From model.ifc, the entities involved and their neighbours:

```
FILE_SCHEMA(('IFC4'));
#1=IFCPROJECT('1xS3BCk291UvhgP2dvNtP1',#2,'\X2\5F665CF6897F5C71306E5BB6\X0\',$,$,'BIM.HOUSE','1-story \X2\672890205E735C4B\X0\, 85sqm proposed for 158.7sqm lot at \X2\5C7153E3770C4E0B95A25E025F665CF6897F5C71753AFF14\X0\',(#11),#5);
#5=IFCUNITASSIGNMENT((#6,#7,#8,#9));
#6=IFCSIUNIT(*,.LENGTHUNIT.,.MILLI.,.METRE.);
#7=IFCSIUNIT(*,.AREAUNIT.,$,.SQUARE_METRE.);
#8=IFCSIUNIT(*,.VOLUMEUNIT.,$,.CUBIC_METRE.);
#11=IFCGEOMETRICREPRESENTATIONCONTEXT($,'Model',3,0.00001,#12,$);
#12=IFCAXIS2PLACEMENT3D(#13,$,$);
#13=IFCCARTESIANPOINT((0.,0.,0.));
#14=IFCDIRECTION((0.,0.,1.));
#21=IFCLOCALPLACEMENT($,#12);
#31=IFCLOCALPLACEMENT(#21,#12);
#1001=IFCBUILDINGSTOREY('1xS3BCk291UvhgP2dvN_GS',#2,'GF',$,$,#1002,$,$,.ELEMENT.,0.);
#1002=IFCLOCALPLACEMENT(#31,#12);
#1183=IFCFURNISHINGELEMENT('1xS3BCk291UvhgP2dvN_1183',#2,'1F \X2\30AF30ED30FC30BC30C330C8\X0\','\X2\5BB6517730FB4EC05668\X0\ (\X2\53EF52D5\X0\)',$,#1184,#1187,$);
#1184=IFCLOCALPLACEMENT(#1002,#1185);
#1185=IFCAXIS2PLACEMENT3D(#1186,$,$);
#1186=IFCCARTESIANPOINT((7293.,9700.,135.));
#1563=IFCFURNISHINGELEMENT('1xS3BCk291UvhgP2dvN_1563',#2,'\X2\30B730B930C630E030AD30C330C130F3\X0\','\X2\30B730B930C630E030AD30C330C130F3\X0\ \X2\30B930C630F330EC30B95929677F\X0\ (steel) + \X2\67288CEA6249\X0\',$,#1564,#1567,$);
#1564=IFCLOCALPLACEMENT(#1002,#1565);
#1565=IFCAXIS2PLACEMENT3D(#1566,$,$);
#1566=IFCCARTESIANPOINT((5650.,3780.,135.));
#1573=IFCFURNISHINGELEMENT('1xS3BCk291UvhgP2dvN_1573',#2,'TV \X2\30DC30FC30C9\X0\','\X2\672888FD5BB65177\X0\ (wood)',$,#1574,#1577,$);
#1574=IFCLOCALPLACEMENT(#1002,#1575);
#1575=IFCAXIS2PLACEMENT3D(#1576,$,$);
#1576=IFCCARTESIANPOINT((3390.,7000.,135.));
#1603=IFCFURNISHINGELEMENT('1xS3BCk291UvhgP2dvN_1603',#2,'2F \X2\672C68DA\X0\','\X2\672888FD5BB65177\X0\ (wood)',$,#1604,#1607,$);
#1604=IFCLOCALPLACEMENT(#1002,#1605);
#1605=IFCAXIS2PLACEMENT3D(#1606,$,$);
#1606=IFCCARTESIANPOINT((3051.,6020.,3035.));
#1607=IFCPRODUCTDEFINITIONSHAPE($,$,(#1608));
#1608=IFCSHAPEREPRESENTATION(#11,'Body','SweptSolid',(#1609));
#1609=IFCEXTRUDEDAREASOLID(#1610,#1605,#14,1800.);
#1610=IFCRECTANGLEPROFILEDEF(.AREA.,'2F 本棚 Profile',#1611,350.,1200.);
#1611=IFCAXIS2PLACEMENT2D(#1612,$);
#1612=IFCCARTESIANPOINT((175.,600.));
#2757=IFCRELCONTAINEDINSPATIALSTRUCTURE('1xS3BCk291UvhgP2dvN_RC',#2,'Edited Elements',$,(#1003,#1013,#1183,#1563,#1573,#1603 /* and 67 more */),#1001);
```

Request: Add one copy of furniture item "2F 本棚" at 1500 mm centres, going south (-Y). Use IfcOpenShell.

```python
import numpy as np
import ifcopenshell
import ifcopenshell.api.geometry
import ifcopenshell.api.root
import ifcopenshell.util.element
import ifcopenshell.util.placement
import ifcopenshell.util.unit

model = ifcopenshell.open("model.ifc")
unit_scale = ifcopenshell.util.unit.calculate_unit_scale(model)


def reuse_history(source, copy):
    """copy_class also copies each property set's owner history, people and application; keep the originals."""
    for rel in copy.IsDefinedBy:
        if rel.is_a("IfcRelDefinesByProperties") and (history := rel.RelatingPropertyDefinition.OwnerHistory):
            rel.RelatingPropertyDefinition.OwnerHistory = source.OwnerHistory
            ifcopenshell.util.element.remove_deep2(model, history)


source = model.by_guid("1xS3BCk291UvhgP2dvN_1603")
base = ifcopenshell.util.placement.get_local_placement(source.ObjectPlacement)
step = np.array([0.0, -1.0, 0.0]) * 1.5 / unit_scale

for i in range(1, 2):
    copy = ifcopenshell.api.root.copy_class(model, product=source)
    copy.Representation = ifcopenshell.util.element.copy_deep(
        model, source.Representation, exclude=["IfcGeometricRepresentationContext", "IfcRepresentationMap"]
    )
    reuse_history(source, copy)
    matrix = base.copy()
    matrix[:3, 3] += i * step
    print("added at", matrix[:3, 3].round(3) + 0.0)
    ifcopenshell.api.geometry.edit_object_placement(model, product=copy, matrix=matrix, is_si=False)

model.write("model_v2.ifc")
```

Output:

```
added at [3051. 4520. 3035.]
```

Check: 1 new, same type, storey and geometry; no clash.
